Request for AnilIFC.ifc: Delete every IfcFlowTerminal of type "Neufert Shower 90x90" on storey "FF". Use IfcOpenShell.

First a look at what the model holds.

```python
import ifcopenshell
import ifcopenshell.util.element

model = ifcopenshell.open("AnilIFC.ifc")
print(model.schema)
storey = next(s for s in model.by_type("IfcBuildingStorey") if s.Name == "FF")
terminals = [e for e in ifcopenshell.util.element.get_decomposition(storey) if e.is_a("IfcFlowTerminal")]
seen = {}
for e in terminals:
    element_type = ifcopenshell.util.element.get_type(e)
    name = element_type.Name if element_type not in (None, e) else None
    seen[name] = seen.get(name, 0) + 1
for name, count in sorted(seen.items(), key=str):
    print(count, "x", name)
```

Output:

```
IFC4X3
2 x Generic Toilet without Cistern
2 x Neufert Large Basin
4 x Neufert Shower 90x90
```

```python
import ifcopenshell
import ifcopenshell.api.root
import ifcopenshell.util.element

model = ifcopenshell.open("AnilIFC.ifc")

storey = next(s for s in model.by_type("IfcBuildingStorey") if s.Name == "FF")
terminals = [e for e in ifcopenshell.util.element.get_decomposition(storey) if e.is_a("IfcFlowTerminal")]
targets = [e for e in terminals if (t := ifcopenshell.util.element.get_type(e)) not in (None, e) and t.Name == "Neufert Shower 90x90"]

for e in targets:
    ifcopenshell.api.root.remove_product(model, product=e)
print(len(targets), "removed")

model.write("AnilIFC_updated.ifc")
```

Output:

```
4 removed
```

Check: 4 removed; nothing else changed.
